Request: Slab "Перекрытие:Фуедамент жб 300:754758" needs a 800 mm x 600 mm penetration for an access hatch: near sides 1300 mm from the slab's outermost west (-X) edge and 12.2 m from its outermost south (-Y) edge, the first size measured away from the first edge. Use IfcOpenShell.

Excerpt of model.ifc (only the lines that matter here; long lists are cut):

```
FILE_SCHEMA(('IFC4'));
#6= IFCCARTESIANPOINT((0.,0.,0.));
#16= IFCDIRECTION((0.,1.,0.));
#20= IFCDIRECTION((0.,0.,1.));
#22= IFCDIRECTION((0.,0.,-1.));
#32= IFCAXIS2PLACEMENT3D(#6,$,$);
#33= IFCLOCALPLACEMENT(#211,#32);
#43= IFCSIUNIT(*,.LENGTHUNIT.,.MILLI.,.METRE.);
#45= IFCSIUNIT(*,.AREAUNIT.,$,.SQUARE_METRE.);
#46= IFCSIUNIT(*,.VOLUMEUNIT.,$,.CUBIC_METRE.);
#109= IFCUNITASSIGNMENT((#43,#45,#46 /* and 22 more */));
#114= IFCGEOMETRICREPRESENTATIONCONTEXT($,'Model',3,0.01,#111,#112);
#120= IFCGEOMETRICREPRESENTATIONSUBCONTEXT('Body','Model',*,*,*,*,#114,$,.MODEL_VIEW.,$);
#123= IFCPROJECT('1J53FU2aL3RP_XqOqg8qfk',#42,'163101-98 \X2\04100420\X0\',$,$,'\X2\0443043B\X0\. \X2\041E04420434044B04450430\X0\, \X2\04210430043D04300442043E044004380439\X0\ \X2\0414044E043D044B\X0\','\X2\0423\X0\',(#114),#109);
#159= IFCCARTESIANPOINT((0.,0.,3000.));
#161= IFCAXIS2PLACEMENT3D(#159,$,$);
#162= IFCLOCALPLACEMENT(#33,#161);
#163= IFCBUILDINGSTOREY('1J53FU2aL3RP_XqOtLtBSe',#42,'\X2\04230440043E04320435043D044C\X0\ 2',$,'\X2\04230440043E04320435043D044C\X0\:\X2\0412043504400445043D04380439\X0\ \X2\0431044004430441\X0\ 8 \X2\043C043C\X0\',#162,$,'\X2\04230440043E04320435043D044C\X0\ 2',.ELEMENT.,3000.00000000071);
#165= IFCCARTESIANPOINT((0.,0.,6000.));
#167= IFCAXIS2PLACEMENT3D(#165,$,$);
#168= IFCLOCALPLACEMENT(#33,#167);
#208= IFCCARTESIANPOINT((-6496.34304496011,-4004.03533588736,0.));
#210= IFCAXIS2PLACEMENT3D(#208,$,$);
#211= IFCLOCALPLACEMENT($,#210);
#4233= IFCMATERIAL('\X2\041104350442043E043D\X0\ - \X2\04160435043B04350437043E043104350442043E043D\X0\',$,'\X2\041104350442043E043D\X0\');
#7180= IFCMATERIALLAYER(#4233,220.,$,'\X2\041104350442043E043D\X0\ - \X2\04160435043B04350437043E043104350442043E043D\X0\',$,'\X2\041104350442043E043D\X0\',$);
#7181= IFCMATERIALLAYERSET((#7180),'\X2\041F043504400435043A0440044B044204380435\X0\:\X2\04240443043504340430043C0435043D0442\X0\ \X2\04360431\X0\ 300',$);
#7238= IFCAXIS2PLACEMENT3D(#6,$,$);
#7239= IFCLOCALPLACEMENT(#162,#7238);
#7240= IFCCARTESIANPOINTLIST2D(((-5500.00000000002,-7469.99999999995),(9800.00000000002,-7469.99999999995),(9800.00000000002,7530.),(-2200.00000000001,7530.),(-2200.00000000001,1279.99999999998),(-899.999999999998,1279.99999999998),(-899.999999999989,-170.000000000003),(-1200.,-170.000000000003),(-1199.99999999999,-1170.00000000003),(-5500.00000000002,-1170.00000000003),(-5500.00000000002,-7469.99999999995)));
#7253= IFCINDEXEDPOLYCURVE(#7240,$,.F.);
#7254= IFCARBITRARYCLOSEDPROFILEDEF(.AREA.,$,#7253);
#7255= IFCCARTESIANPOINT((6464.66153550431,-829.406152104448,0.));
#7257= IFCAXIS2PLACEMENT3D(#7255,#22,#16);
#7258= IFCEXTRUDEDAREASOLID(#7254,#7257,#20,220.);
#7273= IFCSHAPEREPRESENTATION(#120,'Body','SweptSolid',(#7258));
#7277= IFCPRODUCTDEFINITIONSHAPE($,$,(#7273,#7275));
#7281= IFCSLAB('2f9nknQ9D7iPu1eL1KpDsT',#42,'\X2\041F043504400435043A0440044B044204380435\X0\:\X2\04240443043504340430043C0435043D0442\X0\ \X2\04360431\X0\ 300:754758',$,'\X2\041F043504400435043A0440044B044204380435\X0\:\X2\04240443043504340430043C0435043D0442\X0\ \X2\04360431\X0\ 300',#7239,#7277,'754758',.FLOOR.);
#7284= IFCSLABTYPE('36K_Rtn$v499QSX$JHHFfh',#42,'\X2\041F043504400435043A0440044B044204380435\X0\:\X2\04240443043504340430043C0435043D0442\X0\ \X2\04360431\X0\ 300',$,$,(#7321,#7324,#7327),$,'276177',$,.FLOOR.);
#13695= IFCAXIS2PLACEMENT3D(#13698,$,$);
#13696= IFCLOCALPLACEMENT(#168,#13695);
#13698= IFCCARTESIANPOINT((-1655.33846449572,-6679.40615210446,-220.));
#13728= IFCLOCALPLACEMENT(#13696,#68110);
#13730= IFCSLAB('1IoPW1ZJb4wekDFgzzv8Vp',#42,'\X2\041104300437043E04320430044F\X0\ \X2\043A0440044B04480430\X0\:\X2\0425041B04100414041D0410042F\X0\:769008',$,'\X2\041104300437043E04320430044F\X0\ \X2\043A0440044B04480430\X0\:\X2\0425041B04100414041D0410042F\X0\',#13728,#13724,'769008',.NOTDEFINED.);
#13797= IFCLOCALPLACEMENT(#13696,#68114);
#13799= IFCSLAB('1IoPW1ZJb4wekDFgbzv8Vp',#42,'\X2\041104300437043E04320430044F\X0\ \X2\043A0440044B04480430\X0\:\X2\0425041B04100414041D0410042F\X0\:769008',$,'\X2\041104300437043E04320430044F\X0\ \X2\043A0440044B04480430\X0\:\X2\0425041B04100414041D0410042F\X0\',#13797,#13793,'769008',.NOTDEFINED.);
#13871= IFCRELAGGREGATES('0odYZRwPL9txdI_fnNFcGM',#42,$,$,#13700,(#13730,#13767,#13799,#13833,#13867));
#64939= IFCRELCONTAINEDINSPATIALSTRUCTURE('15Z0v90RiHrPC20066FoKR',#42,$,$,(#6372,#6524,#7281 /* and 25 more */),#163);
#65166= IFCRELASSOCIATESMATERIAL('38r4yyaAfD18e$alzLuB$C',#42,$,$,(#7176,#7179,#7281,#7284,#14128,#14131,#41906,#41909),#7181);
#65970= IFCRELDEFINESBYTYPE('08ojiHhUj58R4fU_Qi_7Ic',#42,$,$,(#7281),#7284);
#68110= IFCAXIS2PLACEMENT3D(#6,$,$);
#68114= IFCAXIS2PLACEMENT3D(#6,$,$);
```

```python
import numpy as np
import ifcopenshell
import ifcopenshell.api.feature
import ifcopenshell.api.geometry
import ifcopenshell.api.root
import ifcopenshell.geom
import ifcopenshell.util.placement
import ifcopenshell.util.representation
import ifcopenshell.util.shape
import ifcopenshell.util.unit

model = ifcopenshell.open("model.ifc")
unit_scale = ifcopenshell.util.unit.calculate_unit_scale(model)
settings = ifcopenshell.geom.settings()


def volume(element):
    """Net volume in cubic metres, openings subtracted."""
    shape = ifcopenshell.geom.create_shape(settings, element)
    return ifcopenshell.util.shape.get_volume(shape.geometry)


slab = model.by_guid("2f9nknQ9D7iPu1eL1KpDsT")
before = volume(slab)

# Extent in the slab's own axes, in metres. The edges named are its -X and -Y sides.
slab_shape = ifcopenshell.geom.create_shape(settings, slab)
vertices = ifcopenshell.util.shape.get_vertices(slab_shape.geometry)
x_min, y_min, bottom = vertices.min(axis=0)
top = vertices[:, 2].max()

opening = ifcopenshell.api.root.create_entity(model, ifc_class="IfcOpeningElement", name="Access hatch opening", predefined_type="OPENING")
context = ifcopenshell.util.representation.get_context(model, "Model", "Body", "MODEL_VIEW")
width, depth = 0.8, 0.6
outline = [(0.0, 0.0), (width, 0.0), (width, depth), (0.0, depth), (0.0, 0.0)]
# Overshoot both faces by 50 mm so the cut is clean.
shape = ifcopenshell.api.geometry.add_slab_representation(
    model, context=context, depth=top - bottom + 0.1, polyline=outline
)
ifcopenshell.api.geometry.assign_representation(model, product=opening, representation=shape)

matrix = ifcopenshell.util.placement.get_local_placement(slab.ObjectPlacement)
matrix[:, 3] = matrix @ np.append(np.array([x_min + 1.3, y_min + 12.2, bottom - 0.05]) / unit_scale, 1.0)
ifcopenshell.api.geometry.edit_object_placement(model, product=opening, matrix=matrix, is_si=False)
ifcopenshell.api.feature.add_feature(model, feature=opening, element=slab)

after = volume(slab)

print(f"slab volume {before:.3f} -> {after:.3f} m3")

model.write("model_rev.ifc")
```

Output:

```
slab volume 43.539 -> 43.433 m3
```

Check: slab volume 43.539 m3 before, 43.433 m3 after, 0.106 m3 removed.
